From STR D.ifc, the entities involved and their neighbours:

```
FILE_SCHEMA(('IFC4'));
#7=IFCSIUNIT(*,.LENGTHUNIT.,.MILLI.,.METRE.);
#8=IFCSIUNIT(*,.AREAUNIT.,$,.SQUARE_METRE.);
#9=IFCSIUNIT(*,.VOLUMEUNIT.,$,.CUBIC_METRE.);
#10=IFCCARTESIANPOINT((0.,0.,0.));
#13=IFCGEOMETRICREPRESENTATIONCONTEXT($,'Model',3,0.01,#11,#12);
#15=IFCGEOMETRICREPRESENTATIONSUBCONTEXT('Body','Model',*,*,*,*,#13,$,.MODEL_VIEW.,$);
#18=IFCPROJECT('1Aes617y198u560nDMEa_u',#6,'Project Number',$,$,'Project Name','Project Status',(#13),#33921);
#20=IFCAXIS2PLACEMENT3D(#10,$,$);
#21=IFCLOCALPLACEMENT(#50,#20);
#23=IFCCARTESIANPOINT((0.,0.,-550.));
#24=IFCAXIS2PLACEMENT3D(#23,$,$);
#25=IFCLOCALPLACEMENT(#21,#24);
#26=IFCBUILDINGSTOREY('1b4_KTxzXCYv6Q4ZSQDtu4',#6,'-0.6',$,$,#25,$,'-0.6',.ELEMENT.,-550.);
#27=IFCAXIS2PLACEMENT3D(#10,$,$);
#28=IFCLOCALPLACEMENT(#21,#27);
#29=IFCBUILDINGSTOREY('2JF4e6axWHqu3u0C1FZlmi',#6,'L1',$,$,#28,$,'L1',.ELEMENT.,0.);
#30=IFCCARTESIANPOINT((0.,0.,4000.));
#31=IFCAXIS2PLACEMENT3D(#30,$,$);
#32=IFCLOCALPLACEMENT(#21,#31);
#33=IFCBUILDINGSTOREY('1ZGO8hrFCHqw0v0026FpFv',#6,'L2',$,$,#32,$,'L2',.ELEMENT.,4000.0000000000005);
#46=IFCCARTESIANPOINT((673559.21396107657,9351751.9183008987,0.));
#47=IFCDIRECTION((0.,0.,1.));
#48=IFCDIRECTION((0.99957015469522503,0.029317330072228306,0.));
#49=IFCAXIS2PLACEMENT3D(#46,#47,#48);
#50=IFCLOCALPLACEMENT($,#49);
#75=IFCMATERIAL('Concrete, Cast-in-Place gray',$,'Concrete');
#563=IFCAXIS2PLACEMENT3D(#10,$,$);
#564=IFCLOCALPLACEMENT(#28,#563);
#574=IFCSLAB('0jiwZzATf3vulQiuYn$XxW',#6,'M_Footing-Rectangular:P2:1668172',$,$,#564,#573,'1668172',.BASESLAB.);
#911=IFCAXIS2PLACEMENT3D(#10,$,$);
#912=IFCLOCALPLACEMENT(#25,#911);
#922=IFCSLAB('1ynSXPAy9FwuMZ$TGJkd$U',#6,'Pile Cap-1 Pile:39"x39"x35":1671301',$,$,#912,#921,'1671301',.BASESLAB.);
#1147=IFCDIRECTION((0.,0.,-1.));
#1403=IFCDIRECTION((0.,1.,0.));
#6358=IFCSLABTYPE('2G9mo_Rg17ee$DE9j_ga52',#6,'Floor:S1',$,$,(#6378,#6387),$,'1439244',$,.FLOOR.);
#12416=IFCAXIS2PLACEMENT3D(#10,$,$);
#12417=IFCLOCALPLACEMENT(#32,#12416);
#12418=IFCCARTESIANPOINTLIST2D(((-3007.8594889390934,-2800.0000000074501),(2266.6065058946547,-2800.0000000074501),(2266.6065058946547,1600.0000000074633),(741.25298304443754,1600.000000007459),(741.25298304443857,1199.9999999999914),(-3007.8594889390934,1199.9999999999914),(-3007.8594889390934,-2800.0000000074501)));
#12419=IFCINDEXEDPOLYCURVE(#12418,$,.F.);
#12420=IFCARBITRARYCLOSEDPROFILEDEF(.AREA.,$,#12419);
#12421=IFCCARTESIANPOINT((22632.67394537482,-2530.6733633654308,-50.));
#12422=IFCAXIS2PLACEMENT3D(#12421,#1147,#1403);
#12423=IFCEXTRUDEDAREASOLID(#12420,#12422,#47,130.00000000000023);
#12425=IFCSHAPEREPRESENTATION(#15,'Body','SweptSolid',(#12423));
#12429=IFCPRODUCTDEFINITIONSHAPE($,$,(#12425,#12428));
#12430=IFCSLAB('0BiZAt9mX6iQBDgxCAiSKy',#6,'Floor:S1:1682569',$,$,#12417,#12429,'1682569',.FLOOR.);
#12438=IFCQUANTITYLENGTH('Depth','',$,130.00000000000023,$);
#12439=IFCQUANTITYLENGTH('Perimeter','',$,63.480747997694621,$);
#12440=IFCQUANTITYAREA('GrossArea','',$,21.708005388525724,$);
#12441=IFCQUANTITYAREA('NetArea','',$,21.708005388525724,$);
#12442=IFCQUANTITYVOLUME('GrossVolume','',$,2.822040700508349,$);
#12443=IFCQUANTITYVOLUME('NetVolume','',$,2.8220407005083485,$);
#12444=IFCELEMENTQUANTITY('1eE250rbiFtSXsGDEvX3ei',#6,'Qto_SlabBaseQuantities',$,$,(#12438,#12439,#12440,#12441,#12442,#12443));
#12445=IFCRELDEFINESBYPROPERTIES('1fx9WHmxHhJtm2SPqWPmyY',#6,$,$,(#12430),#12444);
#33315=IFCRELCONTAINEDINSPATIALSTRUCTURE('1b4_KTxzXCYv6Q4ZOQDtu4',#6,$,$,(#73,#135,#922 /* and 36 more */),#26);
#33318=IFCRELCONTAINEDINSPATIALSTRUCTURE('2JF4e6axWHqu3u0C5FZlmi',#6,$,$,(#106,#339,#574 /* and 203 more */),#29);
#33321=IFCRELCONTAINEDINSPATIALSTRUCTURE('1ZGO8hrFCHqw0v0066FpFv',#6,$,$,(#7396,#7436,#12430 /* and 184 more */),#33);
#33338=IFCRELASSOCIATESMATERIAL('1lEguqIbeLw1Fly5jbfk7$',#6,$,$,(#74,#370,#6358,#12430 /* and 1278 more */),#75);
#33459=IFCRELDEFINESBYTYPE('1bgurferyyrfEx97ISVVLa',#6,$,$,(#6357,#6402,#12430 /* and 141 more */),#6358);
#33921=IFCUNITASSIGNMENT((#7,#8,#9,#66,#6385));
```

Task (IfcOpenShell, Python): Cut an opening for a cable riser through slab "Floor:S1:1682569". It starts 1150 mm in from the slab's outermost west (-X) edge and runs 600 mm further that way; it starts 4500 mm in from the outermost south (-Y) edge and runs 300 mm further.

```python
import numpy as np
import ifcopenshell
import ifcopenshell.api.feature
import ifcopenshell.api.geometry
import ifcopenshell.api.pset
import ifcopenshell.api.root
import ifcopenshell.geom
import ifcopenshell.util.element
import ifcopenshell.util.placement
import ifcopenshell.util.representation
import ifcopenshell.util.shape
import ifcopenshell.util.unit

model = ifcopenshell.open("STR D.ifc")
unit_scale = ifcopenshell.util.unit.calculate_unit_scale(model)
area_scale = ifcopenshell.util.unit.calculate_unit_scale(model, "AREAUNIT")
volume_scale = ifcopenshell.util.unit.calculate_unit_scale(model, "VOLUMEUNIT")
settings = ifcopenshell.geom.settings()


def volume(element):
    """Net volume in cubic metres, openings subtracted."""
    shape = ifcopenshell.geom.create_shape(settings, element)
    return ifcopenshell.util.shape.get_volume(shape.geometry)


slab = model.by_id(12430)
before = volume(slab)

# Extent in the slab's own axes, in metres. The edges named are its -X and -Y sides.
slab_shape = ifcopenshell.geom.create_shape(settings, slab)
vertices = ifcopenshell.util.shape.get_vertices(slab_shape.geometry)
x_min, y_min, bottom = vertices.min(axis=0)
top = vertices[:, 2].max()

opening = ifcopenshell.api.root.create_entity(model, ifc_class="IfcOpeningElement", name="Cable riser opening", predefined_type="OPENING")
context = ifcopenshell.util.representation.get_context(model, "Model", "Body", "MODEL_VIEW")
width, depth = 0.6, 0.3
outline = [(0.0, 0.0), (width, 0.0), (width, depth), (0.0, depth), (0.0, 0.0)]
# Overshoot both faces by 50 mm so the cut is clean.
shape = ifcopenshell.api.geometry.add_slab_representation(
    model, context=context, depth=top - bottom + 0.1, polyline=outline
)
ifcopenshell.api.geometry.assign_representation(model, product=opening, representation=shape)

matrix = ifcopenshell.util.placement.get_local_placement(slab.ObjectPlacement)
matrix[:, 3] = matrix @ np.append(np.array([x_min + 1.15, y_min + 4.5, bottom - 0.05]) / unit_scale, 1.0)
ifcopenshell.api.geometry.edit_object_placement(model, product=opening, matrix=matrix, is_si=False)
ifcopenshell.api.feature.add_feature(model, feature=opening, element=slab)

after = volume(slab)

# Update the slab's stored quantities.
qto = model.by_id(ifcopenshell.util.element.get_pset(slab, "Qto_SlabBaseQuantities", should_inherit=False)["id"])
ifcopenshell.api.pset.edit_qto(model, qto=qto, properties={
    "NetArea": after / (top - bottom) / area_scale,
    "NetVolume": after / volume_scale,
})

print(f"slab volume {before:.3f} -> {after:.3f} m3")

model.write("STR D_updated.ifc")
```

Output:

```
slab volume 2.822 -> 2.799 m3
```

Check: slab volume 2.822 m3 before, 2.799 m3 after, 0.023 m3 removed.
